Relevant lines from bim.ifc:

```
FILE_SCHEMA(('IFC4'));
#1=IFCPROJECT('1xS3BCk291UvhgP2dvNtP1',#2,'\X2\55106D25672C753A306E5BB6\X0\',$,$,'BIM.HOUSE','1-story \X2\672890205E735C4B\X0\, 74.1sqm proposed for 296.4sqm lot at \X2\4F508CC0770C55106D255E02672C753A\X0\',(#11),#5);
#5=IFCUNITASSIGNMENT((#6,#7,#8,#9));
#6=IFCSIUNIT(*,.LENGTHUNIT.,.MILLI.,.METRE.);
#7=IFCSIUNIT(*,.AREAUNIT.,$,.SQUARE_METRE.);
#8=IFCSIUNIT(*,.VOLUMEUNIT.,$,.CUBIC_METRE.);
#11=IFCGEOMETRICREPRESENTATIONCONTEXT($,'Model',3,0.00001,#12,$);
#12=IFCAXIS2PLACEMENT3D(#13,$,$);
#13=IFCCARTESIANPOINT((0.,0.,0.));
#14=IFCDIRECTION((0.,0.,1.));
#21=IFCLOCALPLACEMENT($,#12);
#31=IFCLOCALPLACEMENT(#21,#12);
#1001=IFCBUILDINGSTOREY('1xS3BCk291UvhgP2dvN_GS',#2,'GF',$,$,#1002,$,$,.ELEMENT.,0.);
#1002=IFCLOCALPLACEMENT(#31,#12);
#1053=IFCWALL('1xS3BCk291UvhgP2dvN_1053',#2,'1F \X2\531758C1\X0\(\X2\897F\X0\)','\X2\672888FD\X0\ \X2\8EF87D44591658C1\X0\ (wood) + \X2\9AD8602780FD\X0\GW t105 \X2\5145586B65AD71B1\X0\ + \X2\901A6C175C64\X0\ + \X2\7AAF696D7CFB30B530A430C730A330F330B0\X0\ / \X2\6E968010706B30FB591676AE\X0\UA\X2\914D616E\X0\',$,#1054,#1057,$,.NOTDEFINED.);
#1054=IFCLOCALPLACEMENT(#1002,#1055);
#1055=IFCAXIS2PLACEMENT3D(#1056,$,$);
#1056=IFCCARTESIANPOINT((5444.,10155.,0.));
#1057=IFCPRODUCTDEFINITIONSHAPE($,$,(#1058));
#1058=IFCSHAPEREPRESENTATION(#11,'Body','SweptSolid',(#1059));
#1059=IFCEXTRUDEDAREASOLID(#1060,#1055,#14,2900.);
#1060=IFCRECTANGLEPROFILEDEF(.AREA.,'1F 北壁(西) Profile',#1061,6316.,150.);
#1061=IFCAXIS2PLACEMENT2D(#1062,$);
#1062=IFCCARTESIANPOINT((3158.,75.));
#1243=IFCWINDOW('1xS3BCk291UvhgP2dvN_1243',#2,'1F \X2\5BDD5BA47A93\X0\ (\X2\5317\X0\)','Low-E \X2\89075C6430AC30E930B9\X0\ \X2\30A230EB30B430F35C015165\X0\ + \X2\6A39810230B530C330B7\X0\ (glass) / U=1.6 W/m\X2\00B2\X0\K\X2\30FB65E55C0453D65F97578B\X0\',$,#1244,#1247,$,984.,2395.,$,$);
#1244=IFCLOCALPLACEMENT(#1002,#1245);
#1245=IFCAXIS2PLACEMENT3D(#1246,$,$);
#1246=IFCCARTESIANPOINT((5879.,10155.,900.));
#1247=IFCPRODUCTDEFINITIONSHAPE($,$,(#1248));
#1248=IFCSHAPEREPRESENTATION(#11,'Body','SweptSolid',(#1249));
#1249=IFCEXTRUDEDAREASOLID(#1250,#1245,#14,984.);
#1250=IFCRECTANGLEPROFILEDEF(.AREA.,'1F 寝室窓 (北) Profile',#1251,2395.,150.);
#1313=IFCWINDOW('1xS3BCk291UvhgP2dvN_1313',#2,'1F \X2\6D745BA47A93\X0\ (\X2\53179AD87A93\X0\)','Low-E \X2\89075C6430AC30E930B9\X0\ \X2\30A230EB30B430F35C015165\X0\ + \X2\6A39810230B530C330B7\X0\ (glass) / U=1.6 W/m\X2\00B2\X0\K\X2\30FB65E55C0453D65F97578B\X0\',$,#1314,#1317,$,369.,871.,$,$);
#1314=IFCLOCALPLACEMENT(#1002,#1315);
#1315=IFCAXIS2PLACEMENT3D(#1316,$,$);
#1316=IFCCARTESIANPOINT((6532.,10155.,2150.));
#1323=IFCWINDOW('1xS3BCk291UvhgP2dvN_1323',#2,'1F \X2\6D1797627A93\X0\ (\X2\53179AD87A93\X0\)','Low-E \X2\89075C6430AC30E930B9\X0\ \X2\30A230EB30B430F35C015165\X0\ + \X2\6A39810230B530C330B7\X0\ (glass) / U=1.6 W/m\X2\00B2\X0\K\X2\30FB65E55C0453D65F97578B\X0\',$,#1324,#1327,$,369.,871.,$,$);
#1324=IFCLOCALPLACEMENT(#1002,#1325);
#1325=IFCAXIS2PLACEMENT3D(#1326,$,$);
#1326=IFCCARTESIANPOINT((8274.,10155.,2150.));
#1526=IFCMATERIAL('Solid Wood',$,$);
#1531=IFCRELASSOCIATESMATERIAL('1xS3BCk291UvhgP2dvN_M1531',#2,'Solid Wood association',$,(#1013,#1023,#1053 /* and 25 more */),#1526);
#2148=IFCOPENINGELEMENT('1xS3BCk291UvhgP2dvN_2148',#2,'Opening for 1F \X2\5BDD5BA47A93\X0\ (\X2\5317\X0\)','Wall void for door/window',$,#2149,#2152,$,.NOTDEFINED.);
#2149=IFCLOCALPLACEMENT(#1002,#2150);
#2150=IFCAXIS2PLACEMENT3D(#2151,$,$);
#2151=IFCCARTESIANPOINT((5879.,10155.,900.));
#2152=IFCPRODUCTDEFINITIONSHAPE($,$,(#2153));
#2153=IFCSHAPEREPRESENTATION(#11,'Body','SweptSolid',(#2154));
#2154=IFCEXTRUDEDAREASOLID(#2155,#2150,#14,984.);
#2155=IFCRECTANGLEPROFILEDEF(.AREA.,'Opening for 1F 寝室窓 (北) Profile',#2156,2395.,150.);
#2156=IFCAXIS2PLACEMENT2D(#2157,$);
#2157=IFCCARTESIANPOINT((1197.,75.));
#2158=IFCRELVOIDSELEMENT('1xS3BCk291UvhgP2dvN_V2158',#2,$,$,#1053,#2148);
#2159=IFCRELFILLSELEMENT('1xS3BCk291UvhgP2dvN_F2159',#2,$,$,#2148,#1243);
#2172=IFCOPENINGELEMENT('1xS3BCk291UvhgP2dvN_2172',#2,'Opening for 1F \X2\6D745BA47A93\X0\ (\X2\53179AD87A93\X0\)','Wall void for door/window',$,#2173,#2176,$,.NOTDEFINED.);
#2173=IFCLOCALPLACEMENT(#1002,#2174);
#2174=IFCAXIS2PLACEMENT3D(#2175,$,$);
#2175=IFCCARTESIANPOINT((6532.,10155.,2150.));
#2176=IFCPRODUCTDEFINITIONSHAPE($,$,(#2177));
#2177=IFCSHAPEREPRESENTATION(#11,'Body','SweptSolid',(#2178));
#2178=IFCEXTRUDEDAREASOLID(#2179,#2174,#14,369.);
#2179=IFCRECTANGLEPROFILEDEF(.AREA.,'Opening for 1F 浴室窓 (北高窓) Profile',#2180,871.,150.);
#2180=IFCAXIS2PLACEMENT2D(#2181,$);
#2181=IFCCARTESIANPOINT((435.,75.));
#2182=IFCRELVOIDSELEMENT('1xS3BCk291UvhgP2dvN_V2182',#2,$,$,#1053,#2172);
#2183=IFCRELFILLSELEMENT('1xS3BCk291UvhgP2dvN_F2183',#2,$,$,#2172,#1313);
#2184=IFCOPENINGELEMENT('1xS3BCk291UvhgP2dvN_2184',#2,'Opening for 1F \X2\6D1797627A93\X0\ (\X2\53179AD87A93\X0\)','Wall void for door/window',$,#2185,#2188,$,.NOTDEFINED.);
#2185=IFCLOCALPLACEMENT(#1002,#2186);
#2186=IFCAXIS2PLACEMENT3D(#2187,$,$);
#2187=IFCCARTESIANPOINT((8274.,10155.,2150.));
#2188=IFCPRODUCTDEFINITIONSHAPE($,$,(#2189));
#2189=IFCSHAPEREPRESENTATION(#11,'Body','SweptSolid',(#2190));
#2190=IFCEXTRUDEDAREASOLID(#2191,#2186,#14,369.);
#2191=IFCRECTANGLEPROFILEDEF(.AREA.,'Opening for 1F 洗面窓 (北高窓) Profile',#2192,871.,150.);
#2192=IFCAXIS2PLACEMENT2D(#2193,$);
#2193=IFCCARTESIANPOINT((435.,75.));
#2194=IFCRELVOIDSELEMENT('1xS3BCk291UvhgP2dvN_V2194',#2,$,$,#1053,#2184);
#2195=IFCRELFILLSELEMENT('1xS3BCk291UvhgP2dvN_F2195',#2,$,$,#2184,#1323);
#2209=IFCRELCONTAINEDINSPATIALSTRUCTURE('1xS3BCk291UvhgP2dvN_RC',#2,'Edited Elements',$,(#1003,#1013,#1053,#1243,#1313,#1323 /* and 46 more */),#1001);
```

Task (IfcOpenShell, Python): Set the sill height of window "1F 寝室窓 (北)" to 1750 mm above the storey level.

```python
import numpy as np
import ifcopenshell
import ifcopenshell.api.geometry
import ifcopenshell.geom
import ifcopenshell.util.element
import ifcopenshell.util.placement
import ifcopenshell.util.shape
import ifcopenshell.util.unit

model = ifcopenshell.open("bim.ifc")
unit_scale = ifcopenshell.util.unit.calculate_unit_scale(model)

window = model.by_guid("1xS3BCk291UvhgP2dvN_1243")
opening = window.FillsVoids[0].RelatingOpeningElement
storey = ifcopenshell.util.element.get_container(window, ifc_class="IfcBuildingStorey")
level = ifcopenshell.util.placement.get_local_placement(storey.ObjectPlacement)[2, 3]

# The opening's origin need not be at the sill, so measure its lowest point.
shape = ifcopenshell.geom.create_shape(ifcopenshell.geom.settings(), opening)
bottom = ifcopenshell.util.shape.get_shape_bottom_elevation(shape, shape.geometry) / unit_scale
dz = level + 1750.0 - bottom

shift = np.array([0.0, 0.0, dz])
# The window is not placed relative to its opening, so move both.
for product in (opening, window):
    matrix = ifcopenshell.util.placement.get_local_placement(product.ObjectPlacement)
    matrix[:3, 3] += shift
    ifcopenshell.api.geometry.edit_object_placement(model, product=product, matrix=matrix, is_si=False)

print(f"moved by {dz * unit_scale:+.3f} m")

model.write("bim_edited.ifc")
```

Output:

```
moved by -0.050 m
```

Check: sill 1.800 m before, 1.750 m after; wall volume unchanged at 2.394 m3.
